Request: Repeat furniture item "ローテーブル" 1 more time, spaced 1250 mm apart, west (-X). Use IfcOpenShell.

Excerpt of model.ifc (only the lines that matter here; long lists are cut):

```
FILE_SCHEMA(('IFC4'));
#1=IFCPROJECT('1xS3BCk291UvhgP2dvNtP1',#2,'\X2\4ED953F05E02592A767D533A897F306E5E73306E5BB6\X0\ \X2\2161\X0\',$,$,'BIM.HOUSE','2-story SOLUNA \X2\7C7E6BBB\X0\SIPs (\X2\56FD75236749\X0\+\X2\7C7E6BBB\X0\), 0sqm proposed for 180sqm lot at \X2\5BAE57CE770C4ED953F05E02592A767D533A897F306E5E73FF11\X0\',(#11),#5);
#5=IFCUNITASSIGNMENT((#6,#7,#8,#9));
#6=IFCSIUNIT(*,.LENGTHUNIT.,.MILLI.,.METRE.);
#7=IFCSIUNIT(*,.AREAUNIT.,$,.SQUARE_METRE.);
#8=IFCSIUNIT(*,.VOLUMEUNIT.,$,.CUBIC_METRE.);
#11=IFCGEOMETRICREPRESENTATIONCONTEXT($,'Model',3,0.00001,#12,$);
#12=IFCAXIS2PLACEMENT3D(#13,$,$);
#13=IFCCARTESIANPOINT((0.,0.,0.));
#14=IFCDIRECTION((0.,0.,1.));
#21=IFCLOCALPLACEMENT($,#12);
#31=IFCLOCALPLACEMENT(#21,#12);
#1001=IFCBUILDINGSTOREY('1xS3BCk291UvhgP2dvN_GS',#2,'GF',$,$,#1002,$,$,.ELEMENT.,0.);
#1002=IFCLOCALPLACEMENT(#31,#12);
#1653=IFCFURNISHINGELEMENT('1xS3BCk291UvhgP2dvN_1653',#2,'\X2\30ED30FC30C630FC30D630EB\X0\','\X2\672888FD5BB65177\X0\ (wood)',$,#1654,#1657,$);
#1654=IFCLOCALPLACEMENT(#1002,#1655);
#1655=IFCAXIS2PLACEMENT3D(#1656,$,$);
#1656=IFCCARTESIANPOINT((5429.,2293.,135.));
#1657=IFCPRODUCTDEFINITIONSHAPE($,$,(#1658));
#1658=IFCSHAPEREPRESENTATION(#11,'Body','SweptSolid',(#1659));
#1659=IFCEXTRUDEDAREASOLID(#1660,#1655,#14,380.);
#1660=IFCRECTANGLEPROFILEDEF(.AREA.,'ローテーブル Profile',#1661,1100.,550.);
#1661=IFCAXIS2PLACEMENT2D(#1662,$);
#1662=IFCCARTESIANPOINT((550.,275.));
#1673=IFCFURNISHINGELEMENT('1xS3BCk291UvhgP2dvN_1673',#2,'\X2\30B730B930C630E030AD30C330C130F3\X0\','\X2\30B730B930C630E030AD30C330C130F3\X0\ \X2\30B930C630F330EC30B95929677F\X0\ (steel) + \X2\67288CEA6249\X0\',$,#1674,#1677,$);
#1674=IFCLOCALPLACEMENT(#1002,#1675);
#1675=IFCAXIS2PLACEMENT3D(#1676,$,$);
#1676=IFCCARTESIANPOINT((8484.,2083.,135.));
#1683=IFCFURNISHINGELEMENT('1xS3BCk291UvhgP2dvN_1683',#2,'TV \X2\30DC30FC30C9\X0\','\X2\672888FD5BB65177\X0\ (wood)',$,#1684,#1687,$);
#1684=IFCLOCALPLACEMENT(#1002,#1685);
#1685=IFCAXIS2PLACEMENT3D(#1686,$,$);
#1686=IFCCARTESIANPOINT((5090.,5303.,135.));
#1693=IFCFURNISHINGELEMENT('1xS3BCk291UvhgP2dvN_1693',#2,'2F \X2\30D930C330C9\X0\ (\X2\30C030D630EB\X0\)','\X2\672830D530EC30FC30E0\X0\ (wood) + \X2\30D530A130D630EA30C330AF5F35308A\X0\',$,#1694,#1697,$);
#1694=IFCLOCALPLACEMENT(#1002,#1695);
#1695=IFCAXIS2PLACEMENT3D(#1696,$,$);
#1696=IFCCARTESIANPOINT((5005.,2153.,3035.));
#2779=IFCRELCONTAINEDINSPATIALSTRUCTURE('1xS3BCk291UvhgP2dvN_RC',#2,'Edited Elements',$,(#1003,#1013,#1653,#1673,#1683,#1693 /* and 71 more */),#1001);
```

```python
import numpy as np
import ifcopenshell
import ifcopenshell.api.geometry
import ifcopenshell.api.root
import ifcopenshell.util.element
import ifcopenshell.util.placement
import ifcopenshell.util.unit

model = ifcopenshell.open("model.ifc")
unit_scale = ifcopenshell.util.unit.calculate_unit_scale(model)


def reuse_history(source, copy):
    """copy_class also copies each property set's owner history, people and application; keep the originals."""
    for rel in copy.IsDefinedBy:
        if rel.is_a("IfcRelDefinesByProperties") and (history := rel.RelatingPropertyDefinition.OwnerHistory):
            rel.RelatingPropertyDefinition.OwnerHistory = source.OwnerHistory
            ifcopenshell.util.element.remove_deep2(model, history)


source = model.by_guid("1xS3BCk291UvhgP2dvN_1653")
base = ifcopenshell.util.placement.get_local_placement(source.ObjectPlacement)
step = np.array([-1.0, 0.0, 0.0]) * 1.25 / unit_scale

for i in range(1, 2):
    copy = ifcopenshell.api.root.copy_class(model, product=source)
    copy.Representation = ifcopenshell.util.element.copy_deep(
        model, source.Representation, exclude=["IfcGeometricRepresentationContext", "IfcRepresentationMap"]
    )
    reuse_history(source, copy)
    matrix = base.copy()
    matrix[:3, 3] += i * step
    print("added at", matrix[:3, 3].round(3) + 0.0)
    ifcopenshell.api.geometry.edit_object_placement(model, product=copy, matrix=matrix, is_si=False)

model.write("model_v2.ifc")
```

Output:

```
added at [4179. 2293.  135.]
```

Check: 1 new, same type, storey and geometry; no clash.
